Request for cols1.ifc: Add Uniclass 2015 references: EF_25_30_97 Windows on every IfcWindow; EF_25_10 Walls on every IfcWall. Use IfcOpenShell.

First a look at what the model holds.

```python
import ifcopenshell

model = ifcopenshell.open("cols1.ifc")
print(model.schema)
print("classifications:", [c.Name for c in model.by_type("IfcClassification")])
for ifc_class in ("IfcDoor", "IfcRoof", "IfcStair", "IfcWall", "IfcWindow"):
    print(ifc_class, len(model.by_type(ifc_class)))
```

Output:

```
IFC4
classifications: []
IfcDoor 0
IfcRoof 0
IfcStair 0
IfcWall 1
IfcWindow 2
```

```python
import ifcopenshell
import ifcopenshell.api.classification

model = ifcopenshell.open("cols1.ifc")

system = ifcopenshell.api.classification.add_classification(model, classification="Uniclass 2015")

codes = {
    "IfcWindow": ("EF_25_30_97", "Windows"),
    "IfcWall": ("EF_25_10", "Walls"),
}
for ifc_class, (code, name) in codes.items():
    products = model.by_type(ifc_class)
    ifcopenshell.api.classification.add_reference(
        model, products=products, classification=system, identification=code, name=name
    )
    print(code, len(products))

model.write("cols1-out.ifc")
```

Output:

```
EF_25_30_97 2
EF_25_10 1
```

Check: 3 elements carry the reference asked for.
